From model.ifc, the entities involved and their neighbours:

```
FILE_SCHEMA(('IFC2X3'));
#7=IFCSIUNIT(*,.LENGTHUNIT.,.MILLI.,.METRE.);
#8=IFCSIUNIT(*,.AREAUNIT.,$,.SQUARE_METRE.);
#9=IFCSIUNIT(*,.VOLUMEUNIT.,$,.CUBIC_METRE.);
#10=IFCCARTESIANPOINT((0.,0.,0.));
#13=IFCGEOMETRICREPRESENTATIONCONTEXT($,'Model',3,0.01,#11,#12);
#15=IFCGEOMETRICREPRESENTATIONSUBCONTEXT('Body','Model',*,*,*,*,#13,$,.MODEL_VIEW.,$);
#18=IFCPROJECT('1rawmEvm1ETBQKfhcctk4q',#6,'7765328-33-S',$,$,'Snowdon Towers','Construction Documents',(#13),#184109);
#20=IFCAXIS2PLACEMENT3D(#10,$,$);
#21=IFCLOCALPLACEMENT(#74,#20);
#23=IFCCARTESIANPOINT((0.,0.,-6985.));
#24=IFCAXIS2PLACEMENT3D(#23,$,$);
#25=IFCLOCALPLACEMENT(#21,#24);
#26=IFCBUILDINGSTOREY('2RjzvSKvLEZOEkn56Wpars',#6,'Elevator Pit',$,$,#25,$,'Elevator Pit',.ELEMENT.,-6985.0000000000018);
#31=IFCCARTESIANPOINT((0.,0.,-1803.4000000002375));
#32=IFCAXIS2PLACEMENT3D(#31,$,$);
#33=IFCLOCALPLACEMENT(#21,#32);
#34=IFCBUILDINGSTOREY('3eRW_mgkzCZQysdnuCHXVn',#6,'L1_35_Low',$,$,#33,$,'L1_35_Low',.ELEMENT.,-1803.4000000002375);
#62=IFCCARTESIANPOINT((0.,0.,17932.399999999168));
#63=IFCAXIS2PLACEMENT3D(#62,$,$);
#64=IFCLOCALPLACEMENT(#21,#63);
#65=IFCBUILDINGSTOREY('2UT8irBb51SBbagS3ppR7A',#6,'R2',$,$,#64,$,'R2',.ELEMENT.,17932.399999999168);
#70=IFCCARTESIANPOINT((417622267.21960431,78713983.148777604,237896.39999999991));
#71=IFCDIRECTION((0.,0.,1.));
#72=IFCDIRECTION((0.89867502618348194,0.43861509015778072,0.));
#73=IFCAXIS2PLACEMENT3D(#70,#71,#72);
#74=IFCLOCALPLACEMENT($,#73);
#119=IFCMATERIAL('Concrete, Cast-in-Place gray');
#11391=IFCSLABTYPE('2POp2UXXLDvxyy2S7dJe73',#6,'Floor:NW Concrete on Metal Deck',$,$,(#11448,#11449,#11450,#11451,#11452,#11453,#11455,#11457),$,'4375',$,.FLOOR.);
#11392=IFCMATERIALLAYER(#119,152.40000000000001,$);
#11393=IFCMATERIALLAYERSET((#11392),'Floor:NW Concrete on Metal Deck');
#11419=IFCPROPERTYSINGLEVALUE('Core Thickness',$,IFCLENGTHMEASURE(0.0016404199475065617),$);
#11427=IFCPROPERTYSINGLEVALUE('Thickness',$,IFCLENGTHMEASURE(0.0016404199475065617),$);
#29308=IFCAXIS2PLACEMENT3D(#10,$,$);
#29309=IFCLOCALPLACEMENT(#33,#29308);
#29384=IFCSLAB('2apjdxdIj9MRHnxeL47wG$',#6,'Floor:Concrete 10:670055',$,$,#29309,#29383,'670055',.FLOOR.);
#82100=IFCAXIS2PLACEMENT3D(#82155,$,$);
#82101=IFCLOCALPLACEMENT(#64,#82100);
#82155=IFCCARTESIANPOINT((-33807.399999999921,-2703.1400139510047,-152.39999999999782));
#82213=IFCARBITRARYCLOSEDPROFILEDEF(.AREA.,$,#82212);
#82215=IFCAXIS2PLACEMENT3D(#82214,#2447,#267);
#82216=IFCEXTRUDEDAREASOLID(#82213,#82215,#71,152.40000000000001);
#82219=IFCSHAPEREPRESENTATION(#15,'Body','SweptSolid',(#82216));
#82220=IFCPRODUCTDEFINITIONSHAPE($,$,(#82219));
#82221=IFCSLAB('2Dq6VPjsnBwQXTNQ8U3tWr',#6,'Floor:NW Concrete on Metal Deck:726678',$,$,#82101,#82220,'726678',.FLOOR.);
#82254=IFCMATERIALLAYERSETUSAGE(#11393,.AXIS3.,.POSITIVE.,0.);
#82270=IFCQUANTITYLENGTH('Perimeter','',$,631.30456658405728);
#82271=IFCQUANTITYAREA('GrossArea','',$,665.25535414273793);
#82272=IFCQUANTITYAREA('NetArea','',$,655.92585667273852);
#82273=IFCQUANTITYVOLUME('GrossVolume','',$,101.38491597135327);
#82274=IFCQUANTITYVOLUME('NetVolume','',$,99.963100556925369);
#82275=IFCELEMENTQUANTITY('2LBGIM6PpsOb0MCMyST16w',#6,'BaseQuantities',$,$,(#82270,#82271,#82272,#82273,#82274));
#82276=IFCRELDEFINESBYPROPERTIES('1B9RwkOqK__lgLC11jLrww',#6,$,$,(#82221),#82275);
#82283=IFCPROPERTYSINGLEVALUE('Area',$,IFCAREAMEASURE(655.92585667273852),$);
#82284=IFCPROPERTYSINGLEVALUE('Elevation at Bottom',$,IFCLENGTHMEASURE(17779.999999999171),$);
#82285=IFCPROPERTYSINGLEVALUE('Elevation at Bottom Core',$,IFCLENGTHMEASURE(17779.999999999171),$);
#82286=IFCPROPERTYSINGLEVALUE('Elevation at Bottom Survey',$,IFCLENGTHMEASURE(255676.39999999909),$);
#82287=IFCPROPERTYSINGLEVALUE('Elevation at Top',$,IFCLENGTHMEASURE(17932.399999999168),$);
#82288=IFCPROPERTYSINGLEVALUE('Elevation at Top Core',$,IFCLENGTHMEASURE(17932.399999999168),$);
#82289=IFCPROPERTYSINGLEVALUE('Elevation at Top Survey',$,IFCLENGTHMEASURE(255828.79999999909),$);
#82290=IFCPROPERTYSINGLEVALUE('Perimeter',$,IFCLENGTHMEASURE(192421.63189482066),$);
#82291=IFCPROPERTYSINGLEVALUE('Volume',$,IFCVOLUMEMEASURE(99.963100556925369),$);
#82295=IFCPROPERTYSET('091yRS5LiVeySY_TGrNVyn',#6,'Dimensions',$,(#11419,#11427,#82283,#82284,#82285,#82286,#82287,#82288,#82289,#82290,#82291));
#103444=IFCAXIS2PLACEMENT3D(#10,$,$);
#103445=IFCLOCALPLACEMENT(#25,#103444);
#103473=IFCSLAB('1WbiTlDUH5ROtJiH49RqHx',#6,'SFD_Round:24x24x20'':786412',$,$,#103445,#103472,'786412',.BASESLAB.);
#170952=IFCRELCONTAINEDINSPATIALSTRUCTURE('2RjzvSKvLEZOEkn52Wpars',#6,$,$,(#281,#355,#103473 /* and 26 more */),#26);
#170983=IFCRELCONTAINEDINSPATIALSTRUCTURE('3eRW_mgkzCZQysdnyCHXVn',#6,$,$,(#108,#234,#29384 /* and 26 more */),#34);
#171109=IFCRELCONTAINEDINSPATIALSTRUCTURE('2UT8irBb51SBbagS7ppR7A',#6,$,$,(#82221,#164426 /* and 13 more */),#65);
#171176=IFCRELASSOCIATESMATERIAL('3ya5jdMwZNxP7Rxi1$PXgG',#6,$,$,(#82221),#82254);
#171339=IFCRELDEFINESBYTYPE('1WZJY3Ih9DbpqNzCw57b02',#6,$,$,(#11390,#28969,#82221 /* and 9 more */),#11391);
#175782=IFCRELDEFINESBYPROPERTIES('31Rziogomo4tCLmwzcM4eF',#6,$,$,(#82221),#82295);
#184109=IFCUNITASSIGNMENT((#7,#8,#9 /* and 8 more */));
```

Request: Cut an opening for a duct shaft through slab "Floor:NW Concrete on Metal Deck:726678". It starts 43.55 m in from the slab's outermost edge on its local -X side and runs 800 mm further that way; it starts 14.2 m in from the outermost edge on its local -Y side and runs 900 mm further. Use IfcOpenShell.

```python
import numpy as np
import ifcopenshell
import ifcopenshell.api.feature
import ifcopenshell.api.geometry
import ifcopenshell.api.pset
import ifcopenshell.api.root
import ifcopenshell.geom
import ifcopenshell.util.element
import ifcopenshell.util.placement
import ifcopenshell.util.representation
import ifcopenshell.util.shape
import ifcopenshell.util.unit

model = ifcopenshell.open("model.ifc")
unit_scale = ifcopenshell.util.unit.calculate_unit_scale(model)
area_scale = ifcopenshell.util.unit.calculate_unit_scale(model, "AREAUNIT")
volume_scale = ifcopenshell.util.unit.calculate_unit_scale(model, "VOLUMEUNIT")
settings = ifcopenshell.geom.settings()


def volume(element):
    """Net volume in cubic metres, openings subtracted."""
    shape = ifcopenshell.geom.create_shape(settings, element)
    return ifcopenshell.util.shape.get_volume(shape.geometry)


slab = model.by_guid("2Dq6VPjsnBwQXTNQ8U3tWr")
before = volume(slab)

# Extent in the slab's own axes, in metres. The edges named are its -X and -Y sides.
slab_shape = ifcopenshell.geom.create_shape(settings, slab)
vertices = ifcopenshell.util.shape.get_vertices(slab_shape.geometry)
x_min, y_min, bottom = vertices.min(axis=0)
top = vertices[:, 2].max()

opening = ifcopenshell.api.root.create_entity(model, ifc_class="IfcOpeningElement", name="Duct shaft opening")
context = ifcopenshell.util.representation.get_context(model, "Model", "Body", "MODEL_VIEW")
width, depth = 0.8, 0.9
outline = [(0.0, 0.0), (width, 0.0), (width, depth), (0.0, depth), (0.0, 0.0)]
# Overshoot both faces by 50 mm so the cut is clean.
shape = ifcopenshell.api.geometry.add_slab_representation(
    model, context=context, depth=top - bottom + 0.1, polyline=outline
)
ifcopenshell.api.geometry.assign_representation(model, product=opening, representation=shape)

matrix = ifcopenshell.util.placement.get_local_placement(slab.ObjectPlacement)
matrix[:, 3] = matrix @ np.append(np.array([x_min + 43.55, y_min + 14.2, bottom - 0.05]) / unit_scale, 1.0)
ifcopenshell.api.geometry.edit_object_placement(model, product=opening, matrix=matrix, is_si=False)
ifcopenshell.api.feature.add_feature(model, feature=opening, element=slab)

after = volume(slab)

# Update the slab's stored quantities.
qto = model.by_id(ifcopenshell.util.element.get_pset(slab, "BaseQuantities", should_inherit=False)["id"])
ifcopenshell.api.pset.edit_qto(model, qto=qto, properties={
    "NetArea": after / (top - bottom) / area_scale,
    "NetVolume": after / volume_scale,
})
pset = model.by_id(ifcopenshell.util.element.get_pset(slab, "Dimensions", should_inherit=False)["id"])
ifcopenshell.api.pset.edit_pset(model, pset=pset, properties={
    "Area": model.create_entity("IfcAreaMeasure", after / (top - bottom) / area_scale),
    "Volume": model.create_entity("IfcVolumeMeasure", after / volume_scale),
})

print(f"slab volume {before:.3f} -> {after:.3f} m3")

model.write("model_updated.ifc")
```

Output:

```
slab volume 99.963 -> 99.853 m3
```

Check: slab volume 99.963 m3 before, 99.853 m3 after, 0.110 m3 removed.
